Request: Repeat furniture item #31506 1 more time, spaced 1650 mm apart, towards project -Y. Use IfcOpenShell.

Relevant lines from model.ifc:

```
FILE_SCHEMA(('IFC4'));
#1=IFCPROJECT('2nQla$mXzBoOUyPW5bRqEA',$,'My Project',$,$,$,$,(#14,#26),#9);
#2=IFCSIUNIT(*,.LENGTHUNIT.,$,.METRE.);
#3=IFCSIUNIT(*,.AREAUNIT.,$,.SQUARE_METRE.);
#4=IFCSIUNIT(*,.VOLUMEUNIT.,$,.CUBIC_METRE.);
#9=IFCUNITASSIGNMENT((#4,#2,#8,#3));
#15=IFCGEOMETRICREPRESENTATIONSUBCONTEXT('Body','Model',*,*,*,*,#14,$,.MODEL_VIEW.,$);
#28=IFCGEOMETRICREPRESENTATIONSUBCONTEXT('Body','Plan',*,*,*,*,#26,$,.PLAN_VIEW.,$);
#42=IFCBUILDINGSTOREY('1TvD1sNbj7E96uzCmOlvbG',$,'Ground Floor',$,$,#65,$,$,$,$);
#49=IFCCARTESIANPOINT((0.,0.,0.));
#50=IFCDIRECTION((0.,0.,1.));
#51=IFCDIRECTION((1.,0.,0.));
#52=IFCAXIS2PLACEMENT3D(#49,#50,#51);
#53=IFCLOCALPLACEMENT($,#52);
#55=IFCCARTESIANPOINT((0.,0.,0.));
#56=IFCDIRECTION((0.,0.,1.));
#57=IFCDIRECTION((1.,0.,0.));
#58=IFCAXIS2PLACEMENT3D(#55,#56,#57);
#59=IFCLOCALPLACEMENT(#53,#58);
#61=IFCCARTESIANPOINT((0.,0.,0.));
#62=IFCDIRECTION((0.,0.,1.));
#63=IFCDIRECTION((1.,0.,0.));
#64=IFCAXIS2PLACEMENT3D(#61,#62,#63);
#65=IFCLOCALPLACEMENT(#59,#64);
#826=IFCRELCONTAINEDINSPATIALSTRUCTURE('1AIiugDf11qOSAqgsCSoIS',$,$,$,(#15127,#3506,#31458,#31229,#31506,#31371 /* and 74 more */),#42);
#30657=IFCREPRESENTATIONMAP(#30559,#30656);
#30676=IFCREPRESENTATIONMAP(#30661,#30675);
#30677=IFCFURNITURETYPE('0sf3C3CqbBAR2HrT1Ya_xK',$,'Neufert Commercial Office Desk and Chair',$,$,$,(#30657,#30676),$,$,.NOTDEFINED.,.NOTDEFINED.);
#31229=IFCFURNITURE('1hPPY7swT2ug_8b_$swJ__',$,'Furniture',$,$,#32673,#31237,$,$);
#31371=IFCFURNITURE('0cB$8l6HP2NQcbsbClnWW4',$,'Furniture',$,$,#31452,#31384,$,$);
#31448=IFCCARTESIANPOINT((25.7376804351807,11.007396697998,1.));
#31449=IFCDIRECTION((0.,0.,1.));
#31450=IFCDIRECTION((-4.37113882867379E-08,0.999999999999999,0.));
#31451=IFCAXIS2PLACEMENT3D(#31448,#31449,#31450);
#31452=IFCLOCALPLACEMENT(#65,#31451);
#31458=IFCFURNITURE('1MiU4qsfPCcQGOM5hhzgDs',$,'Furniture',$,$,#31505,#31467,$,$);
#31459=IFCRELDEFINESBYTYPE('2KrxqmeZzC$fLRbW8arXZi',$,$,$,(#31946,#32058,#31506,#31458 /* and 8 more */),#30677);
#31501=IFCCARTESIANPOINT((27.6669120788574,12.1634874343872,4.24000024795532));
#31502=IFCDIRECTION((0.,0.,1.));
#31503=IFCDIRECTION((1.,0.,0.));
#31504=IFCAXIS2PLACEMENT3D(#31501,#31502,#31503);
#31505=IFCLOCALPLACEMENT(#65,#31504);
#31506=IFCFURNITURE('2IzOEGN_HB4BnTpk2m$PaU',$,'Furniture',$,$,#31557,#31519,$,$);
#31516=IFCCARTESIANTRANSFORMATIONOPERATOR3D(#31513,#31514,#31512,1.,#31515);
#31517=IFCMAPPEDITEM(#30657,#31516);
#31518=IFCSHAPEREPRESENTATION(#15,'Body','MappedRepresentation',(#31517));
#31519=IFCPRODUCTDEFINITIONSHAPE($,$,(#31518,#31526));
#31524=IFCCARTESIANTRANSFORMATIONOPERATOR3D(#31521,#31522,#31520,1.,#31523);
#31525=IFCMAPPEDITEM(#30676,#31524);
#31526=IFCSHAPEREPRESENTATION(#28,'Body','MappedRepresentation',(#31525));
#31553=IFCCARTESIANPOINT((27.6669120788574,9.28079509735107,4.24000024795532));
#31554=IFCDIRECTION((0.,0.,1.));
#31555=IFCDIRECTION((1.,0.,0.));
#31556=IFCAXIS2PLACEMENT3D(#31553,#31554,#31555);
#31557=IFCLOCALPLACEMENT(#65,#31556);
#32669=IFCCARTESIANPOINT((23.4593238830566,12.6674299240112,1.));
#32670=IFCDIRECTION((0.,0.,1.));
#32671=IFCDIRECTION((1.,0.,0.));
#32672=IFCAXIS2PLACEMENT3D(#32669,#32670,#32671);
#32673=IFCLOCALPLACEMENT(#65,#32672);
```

```python
import numpy as np
import ifcopenshell
import ifcopenshell.api.geometry
import ifcopenshell.api.root
import ifcopenshell.util.element
import ifcopenshell.util.placement

model = ifcopenshell.open("model.ifc")

source = model.by_id(31506)
base = ifcopenshell.util.placement.get_local_placement(source.ObjectPlacement)
step = np.array([0.0, -1.0, 0.0]) * 1.65

for i in range(1, 2):
    copy = ifcopenshell.api.root.copy_class(model, product=source)
    copy.Representation = ifcopenshell.util.element.copy_deep(
        model, source.Representation, exclude=["IfcGeometricRepresentationContext", "IfcRepresentationMap"]
    )
    matrix = base.copy()
    matrix[:3, 3] += i * step
    print("added at", matrix[:3, 3].round(3) + 0.0)
    ifcopenshell.api.geometry.edit_object_placement(model, product=copy, matrix=matrix, is_si=False)

model.write("model-out.ifc")
```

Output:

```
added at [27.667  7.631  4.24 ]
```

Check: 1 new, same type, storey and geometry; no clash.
